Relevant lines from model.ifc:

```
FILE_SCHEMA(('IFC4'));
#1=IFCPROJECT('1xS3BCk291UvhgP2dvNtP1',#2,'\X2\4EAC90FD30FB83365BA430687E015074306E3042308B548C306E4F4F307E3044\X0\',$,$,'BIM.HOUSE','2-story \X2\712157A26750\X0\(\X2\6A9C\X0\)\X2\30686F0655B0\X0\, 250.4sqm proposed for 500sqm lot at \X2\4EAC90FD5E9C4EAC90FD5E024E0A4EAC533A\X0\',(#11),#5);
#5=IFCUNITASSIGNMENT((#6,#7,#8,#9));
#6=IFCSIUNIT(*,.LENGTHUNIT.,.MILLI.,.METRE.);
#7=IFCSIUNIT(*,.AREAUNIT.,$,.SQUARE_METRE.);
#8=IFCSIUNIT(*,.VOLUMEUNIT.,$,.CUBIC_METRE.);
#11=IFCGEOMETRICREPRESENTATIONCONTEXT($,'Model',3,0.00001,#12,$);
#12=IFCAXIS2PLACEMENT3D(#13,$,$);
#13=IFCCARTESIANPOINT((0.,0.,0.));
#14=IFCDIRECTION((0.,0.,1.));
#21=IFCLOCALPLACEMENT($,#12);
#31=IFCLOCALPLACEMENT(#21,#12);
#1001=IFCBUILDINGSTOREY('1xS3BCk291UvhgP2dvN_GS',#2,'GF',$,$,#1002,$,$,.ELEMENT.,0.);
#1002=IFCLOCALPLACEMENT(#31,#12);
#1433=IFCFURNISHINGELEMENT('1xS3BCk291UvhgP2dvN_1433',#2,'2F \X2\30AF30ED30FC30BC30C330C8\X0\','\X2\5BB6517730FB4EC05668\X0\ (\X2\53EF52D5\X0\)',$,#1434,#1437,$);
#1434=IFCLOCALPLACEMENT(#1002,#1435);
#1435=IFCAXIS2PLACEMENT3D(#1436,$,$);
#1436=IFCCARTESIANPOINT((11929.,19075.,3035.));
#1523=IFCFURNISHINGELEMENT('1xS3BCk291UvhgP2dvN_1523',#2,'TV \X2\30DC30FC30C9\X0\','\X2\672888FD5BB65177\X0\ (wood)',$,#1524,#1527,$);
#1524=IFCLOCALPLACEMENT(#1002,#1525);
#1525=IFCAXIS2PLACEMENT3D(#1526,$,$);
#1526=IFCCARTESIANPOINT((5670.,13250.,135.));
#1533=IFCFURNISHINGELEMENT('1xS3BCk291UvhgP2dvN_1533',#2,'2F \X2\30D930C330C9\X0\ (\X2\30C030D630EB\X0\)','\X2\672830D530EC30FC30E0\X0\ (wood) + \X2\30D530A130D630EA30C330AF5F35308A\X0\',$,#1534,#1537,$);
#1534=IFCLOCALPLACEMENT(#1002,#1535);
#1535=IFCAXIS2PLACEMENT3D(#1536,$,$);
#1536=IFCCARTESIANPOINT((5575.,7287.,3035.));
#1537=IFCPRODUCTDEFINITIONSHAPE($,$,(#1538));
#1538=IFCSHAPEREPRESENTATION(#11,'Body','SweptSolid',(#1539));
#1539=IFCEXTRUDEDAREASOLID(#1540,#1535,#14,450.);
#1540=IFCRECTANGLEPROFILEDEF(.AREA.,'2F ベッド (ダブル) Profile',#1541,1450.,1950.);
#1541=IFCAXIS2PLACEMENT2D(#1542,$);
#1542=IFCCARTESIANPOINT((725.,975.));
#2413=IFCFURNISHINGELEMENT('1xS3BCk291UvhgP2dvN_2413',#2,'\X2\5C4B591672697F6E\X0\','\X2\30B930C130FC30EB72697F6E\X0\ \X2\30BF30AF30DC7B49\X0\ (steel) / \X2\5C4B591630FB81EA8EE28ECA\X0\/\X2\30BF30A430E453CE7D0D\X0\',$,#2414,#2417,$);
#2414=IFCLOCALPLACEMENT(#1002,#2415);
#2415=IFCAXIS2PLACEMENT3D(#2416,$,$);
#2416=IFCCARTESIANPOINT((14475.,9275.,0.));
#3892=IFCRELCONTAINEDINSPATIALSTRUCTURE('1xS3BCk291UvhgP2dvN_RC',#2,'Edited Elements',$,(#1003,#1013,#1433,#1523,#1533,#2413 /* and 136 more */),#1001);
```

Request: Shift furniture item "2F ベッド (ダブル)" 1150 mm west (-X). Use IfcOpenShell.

```python
import ifcopenshell
import ifcopenshell.api.geometry
import ifcopenshell.util.placement
import ifcopenshell.util.unit

model = ifcopenshell.open("model.ifc")
unit_scale = ifcopenshell.util.unit.calculate_unit_scale(model)

item = model.by_id(1533)
matrix = ifcopenshell.util.placement.get_local_placement(item.ObjectPlacement)
matrix[0, 3] -= 1.15 / unit_scale
ifcopenshell.api.geometry.edit_object_placement(model, product=item, matrix=matrix, is_si=False)

print(ifcopenshell.util.placement.get_local_placement(item.ObjectPlacement).round(3) + 0.0)

model.write("model_rev.ifc")
```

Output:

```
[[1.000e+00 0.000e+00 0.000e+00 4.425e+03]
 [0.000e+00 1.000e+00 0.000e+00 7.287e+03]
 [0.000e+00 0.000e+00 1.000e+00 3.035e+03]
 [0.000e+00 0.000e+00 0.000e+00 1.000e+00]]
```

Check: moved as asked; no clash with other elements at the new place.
